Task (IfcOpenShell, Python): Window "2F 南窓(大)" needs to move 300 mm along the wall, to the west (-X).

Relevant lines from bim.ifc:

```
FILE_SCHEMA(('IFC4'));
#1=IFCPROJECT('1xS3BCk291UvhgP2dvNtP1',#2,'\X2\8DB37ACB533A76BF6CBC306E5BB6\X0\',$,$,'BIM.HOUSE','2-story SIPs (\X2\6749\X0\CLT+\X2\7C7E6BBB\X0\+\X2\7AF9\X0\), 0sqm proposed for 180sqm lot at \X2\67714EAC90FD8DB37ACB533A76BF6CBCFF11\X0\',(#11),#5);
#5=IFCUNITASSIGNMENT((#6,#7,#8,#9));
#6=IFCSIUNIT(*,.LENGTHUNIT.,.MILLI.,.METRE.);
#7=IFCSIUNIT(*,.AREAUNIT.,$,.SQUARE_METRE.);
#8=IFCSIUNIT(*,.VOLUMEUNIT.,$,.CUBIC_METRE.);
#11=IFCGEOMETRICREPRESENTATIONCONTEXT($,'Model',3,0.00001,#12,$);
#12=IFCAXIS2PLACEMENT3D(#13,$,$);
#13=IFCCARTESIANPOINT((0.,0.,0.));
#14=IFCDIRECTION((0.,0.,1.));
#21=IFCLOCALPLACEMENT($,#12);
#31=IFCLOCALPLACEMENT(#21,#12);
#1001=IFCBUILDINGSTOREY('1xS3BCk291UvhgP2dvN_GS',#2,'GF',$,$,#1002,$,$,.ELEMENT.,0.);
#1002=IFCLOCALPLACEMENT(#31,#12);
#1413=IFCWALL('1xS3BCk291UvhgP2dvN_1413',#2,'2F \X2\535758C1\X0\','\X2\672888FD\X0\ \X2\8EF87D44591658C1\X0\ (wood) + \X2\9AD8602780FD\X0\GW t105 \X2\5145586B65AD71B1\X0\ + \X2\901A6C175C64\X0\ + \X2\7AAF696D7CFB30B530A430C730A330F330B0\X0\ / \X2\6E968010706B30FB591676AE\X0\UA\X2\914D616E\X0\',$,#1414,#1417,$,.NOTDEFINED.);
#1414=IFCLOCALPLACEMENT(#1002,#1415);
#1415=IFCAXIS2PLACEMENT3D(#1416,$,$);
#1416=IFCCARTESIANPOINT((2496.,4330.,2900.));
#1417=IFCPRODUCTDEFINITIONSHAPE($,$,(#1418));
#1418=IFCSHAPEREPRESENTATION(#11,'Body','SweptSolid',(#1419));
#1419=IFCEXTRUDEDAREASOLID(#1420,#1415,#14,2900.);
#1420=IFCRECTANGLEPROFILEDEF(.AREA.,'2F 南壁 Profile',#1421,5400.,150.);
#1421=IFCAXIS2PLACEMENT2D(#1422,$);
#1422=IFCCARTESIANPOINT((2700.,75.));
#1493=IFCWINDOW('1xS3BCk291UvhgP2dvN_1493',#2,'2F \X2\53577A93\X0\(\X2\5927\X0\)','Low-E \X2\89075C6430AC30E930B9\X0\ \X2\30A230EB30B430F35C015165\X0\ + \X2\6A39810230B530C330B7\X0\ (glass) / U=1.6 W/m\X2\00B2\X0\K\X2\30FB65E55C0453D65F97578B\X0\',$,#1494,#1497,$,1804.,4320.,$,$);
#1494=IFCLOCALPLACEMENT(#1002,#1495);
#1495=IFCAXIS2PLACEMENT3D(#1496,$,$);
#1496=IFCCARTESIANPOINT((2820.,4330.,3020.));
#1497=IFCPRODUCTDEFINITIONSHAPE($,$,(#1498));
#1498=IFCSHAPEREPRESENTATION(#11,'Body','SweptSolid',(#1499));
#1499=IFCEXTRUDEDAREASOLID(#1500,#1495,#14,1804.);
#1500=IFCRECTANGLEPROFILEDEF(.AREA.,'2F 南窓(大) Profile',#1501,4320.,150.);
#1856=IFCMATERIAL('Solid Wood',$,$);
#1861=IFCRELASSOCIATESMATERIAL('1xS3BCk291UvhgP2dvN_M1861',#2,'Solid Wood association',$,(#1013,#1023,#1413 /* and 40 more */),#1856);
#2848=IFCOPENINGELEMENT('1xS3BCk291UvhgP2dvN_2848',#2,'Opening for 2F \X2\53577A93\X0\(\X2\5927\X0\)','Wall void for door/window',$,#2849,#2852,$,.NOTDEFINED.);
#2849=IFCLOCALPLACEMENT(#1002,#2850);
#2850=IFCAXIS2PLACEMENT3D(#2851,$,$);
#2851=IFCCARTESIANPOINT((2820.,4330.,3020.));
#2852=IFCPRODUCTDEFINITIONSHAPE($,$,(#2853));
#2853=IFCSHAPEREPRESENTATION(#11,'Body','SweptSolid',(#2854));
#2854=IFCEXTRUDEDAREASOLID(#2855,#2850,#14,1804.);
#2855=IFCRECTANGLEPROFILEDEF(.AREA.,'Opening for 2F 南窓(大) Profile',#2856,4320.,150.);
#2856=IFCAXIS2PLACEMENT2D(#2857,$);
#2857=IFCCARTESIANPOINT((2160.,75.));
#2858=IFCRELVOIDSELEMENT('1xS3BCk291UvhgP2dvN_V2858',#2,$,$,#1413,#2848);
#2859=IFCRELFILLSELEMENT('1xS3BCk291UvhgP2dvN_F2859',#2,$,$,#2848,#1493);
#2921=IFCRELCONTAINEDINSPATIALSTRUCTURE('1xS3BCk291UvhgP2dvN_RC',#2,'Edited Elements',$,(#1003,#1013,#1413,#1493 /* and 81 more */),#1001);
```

```python
import ifcopenshell
import ifcopenshell.api.geometry
import ifcopenshell.util.placement

model = ifcopenshell.open("bim.ifc")

window = model.by_guid("1xS3BCk291UvhgP2dvN_1493")
opening = window.FillsVoids[0].RelatingOpeningElement
wall = opening.VoidsElements[0].RelatingBuildingElement

wall_matrix = ifcopenshell.util.placement.get_local_placement(wall.ObjectPlacement)
shift = wall_matrix[:3, 0] * -300.0
before = ifcopenshell.util.placement.get_local_placement(window.ObjectPlacement)[:3, 3].copy()

# The window is not placed relative to its opening, so move both.
for product in (opening, window):
    matrix = ifcopenshell.util.placement.get_local_placement(product.ObjectPlacement)
    matrix[:3, 3] += shift
    ifcopenshell.api.geometry.edit_object_placement(model, product=product, matrix=matrix, is_si=False)

after = ifcopenshell.util.placement.get_local_placement(window.ObjectPlacement)[:3, 3]
print("window moved by", (after - before).round(3) + 0.0)

model.write("bim-out.ifc")
```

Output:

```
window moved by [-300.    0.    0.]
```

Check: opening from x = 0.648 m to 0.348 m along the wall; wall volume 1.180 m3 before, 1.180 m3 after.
